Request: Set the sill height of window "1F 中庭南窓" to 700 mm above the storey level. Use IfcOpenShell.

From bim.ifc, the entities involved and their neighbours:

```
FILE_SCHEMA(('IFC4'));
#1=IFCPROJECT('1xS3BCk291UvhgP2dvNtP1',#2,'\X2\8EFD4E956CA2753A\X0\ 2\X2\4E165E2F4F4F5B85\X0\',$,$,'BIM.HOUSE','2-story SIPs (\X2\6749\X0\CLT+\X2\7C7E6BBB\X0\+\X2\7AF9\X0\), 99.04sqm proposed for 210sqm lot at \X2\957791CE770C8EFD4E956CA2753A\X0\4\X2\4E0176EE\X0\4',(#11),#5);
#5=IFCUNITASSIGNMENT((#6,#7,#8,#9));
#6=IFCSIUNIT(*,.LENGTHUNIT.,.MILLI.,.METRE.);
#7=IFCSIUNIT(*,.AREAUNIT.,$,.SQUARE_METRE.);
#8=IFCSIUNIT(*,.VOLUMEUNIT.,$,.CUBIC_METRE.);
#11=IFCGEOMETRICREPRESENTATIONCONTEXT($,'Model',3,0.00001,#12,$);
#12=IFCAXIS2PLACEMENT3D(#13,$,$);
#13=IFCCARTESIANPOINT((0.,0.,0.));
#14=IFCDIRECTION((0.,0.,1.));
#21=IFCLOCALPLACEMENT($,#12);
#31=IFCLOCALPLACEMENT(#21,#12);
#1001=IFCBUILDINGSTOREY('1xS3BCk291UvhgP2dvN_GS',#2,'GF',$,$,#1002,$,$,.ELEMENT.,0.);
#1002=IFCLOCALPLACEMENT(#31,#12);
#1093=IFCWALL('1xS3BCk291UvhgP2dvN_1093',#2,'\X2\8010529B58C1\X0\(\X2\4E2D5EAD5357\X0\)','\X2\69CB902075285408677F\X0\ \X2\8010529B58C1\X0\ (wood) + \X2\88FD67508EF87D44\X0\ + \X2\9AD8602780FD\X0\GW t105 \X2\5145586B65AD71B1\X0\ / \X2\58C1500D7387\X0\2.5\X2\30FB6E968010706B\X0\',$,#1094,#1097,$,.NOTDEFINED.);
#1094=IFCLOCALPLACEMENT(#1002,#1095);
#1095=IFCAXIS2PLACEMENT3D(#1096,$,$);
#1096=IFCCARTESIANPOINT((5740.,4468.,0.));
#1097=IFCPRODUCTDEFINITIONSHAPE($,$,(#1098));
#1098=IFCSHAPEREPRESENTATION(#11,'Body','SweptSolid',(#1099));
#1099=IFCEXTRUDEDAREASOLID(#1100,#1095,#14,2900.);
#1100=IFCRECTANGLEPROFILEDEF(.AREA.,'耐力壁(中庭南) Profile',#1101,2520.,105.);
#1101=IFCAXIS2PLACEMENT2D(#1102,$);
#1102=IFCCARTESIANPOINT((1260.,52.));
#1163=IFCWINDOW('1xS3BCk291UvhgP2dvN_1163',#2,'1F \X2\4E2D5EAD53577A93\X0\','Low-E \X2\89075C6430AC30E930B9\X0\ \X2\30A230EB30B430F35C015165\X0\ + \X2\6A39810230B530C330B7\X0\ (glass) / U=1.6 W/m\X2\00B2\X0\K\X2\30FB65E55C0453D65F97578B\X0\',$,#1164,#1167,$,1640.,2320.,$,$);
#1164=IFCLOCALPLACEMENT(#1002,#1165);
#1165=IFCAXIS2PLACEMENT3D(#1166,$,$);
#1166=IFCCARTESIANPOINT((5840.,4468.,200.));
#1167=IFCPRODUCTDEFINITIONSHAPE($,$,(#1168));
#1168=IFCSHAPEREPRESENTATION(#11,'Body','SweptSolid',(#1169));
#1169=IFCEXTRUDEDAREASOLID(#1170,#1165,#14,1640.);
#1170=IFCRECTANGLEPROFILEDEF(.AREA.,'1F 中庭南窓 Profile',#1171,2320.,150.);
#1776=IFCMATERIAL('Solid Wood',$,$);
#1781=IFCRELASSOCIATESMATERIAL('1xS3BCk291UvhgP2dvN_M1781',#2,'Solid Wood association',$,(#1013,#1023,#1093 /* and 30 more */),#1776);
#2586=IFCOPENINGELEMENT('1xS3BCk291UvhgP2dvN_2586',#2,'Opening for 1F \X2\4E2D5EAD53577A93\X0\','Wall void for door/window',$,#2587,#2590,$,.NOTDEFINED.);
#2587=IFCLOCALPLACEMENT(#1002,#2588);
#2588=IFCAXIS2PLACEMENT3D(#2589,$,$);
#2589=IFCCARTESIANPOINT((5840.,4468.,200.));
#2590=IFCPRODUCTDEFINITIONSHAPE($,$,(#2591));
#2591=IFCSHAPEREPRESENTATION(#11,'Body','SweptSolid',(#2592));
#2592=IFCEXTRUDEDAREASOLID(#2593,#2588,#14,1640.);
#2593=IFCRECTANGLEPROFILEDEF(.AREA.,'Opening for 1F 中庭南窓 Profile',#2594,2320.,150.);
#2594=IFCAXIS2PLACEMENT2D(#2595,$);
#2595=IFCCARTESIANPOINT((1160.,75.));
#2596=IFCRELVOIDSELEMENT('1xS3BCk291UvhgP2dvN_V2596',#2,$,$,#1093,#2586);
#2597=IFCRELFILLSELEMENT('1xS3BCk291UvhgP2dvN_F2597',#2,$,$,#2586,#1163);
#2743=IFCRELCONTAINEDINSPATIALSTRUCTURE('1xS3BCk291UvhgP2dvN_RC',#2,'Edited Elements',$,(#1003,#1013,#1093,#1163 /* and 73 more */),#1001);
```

```python
import numpy as np
import ifcopenshell
import ifcopenshell.api.geometry
import ifcopenshell.geom
import ifcopenshell.util.element
import ifcopenshell.util.placement
import ifcopenshell.util.shape
import ifcopenshell.util.unit

model = ifcopenshell.open("bim.ifc")
unit_scale = ifcopenshell.util.unit.calculate_unit_scale(model)

window = model.by_id(1163)
opening = window.FillsVoids[0].RelatingOpeningElement
storey = ifcopenshell.util.element.get_container(window, ifc_class="IfcBuildingStorey")
level = ifcopenshell.util.placement.get_local_placement(storey.ObjectPlacement)[2, 3]

# The opening's origin need not be at the sill, so measure its lowest point.
shape = ifcopenshell.geom.create_shape(ifcopenshell.geom.settings(), opening)
bottom = ifcopenshell.util.shape.get_shape_bottom_elevation(shape, shape.geometry) / unit_scale
dz = level + 0.7 / unit_scale - bottom

shift = np.array([0.0, 0.0, dz])
# The window is not placed relative to its opening, so move both.
for product in (opening, window):
    matrix = ifcopenshell.util.placement.get_local_placement(product.ObjectPlacement)
    matrix[:3, 3] += shift
    ifcopenshell.api.geometry.edit_object_placement(model, product=product, matrix=matrix, is_si=False)

print(f"moved by {dz * unit_scale:+.3f} m")

model.write("bim_rev.ifc")
```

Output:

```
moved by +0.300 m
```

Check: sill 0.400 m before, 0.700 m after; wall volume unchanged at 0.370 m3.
